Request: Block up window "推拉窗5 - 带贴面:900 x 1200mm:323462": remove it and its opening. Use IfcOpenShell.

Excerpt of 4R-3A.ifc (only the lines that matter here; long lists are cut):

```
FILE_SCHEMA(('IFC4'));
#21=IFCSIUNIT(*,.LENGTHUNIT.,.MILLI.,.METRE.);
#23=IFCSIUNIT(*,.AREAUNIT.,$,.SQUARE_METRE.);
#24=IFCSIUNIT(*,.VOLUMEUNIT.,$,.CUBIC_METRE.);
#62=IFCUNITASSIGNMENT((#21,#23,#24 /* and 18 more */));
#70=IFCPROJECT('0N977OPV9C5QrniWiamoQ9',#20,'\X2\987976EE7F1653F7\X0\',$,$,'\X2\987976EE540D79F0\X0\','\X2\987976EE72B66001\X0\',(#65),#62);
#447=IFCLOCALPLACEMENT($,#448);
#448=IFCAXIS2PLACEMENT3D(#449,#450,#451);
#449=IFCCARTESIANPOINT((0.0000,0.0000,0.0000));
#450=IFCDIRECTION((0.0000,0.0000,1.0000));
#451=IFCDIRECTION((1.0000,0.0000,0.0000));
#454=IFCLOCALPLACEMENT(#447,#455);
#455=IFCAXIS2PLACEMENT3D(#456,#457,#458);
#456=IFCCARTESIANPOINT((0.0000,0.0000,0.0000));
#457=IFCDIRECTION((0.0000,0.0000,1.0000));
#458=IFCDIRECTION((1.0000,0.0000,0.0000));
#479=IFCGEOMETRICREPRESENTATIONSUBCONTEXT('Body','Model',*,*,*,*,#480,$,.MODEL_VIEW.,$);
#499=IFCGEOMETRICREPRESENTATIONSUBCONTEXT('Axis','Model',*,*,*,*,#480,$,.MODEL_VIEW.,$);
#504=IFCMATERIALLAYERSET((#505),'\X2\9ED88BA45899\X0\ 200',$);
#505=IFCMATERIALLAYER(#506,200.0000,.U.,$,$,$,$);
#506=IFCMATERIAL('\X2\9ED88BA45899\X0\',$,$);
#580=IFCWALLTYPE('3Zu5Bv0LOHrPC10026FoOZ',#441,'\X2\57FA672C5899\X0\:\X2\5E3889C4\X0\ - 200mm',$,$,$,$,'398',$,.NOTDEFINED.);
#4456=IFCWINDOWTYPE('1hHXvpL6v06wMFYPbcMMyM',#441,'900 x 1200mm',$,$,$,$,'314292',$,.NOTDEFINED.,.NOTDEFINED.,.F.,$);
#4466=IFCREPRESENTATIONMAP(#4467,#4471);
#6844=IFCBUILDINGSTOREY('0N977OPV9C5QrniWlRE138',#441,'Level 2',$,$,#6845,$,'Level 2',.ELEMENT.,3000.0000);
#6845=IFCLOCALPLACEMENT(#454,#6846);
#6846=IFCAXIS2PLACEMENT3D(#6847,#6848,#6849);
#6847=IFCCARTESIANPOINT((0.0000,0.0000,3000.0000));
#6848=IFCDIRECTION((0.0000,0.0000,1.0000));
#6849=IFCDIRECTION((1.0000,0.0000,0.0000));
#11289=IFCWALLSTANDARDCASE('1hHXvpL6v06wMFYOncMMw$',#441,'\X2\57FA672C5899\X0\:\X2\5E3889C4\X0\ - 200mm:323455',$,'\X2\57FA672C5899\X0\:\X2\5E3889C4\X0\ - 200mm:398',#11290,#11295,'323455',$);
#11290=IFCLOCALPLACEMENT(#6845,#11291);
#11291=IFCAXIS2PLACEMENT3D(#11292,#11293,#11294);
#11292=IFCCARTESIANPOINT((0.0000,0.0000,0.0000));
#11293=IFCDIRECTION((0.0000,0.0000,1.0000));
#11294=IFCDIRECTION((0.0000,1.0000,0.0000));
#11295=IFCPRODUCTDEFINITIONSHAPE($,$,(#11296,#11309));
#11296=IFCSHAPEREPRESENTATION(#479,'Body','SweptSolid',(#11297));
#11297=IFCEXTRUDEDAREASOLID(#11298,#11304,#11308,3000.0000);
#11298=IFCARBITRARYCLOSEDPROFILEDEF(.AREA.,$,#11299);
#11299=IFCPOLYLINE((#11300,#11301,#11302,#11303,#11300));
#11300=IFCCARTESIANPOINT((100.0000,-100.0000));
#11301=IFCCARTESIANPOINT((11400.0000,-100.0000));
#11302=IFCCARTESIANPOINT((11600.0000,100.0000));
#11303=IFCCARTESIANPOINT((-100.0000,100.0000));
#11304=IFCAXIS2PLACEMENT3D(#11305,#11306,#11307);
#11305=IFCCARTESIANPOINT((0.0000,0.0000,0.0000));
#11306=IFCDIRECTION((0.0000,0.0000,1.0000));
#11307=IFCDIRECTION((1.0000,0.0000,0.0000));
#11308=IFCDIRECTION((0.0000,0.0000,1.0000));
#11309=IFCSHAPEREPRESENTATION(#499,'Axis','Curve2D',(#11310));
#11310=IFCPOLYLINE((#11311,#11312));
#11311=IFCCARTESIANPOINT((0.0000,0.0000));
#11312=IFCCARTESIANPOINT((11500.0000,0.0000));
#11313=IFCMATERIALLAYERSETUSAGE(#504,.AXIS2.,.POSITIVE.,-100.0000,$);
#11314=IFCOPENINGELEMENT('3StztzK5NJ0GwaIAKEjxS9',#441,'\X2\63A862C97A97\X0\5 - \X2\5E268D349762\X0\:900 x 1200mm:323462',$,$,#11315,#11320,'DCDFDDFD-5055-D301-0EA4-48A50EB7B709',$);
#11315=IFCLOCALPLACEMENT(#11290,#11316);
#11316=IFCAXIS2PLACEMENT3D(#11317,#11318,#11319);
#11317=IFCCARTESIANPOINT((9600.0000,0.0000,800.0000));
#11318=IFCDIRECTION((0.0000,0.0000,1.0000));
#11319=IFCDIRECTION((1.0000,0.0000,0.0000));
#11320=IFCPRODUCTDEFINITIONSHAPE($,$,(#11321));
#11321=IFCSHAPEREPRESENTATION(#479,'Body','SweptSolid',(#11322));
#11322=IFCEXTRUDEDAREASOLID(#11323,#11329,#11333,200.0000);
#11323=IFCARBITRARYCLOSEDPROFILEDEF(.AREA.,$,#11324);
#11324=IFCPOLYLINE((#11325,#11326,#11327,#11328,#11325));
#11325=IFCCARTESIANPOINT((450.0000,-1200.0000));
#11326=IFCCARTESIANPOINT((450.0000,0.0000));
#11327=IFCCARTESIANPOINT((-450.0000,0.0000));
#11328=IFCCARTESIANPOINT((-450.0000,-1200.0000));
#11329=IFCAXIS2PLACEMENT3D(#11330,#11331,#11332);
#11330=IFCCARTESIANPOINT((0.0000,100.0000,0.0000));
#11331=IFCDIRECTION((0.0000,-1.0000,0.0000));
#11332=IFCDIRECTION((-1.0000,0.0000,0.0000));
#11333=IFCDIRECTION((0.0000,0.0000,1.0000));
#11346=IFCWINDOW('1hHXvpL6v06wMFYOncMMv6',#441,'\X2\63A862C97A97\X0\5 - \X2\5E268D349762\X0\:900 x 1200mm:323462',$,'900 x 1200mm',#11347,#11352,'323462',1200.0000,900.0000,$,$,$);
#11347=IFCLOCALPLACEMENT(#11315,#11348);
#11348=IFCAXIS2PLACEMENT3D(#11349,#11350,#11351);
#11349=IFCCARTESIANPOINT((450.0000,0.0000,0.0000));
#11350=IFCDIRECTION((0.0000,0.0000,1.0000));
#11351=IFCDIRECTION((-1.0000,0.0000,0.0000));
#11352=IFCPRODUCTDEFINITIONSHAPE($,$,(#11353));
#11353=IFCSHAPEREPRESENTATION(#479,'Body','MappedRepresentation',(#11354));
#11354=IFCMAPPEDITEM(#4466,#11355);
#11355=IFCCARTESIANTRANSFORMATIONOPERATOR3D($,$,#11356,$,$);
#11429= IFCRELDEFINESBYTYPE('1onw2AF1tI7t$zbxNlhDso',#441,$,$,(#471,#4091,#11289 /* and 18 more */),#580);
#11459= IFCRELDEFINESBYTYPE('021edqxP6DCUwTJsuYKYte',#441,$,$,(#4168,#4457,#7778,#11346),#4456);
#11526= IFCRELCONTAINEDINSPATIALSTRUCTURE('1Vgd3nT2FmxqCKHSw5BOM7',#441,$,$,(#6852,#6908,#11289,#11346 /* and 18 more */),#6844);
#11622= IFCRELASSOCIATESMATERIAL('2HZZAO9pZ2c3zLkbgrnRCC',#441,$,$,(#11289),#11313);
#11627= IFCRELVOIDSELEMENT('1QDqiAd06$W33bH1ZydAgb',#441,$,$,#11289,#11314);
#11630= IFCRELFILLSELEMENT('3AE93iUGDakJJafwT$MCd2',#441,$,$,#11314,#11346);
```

```python
import ifcopenshell
import ifcopenshell.api.feature
import ifcopenshell.api.root
import ifcopenshell.geom
import ifcopenshell.util.shape

model = ifcopenshell.open("4R-3A.ifc")
settings = ifcopenshell.geom.settings()


def volume(element):
    """Net volume in cubic metres, openings subtracted."""
    shape = ifcopenshell.geom.create_shape(settings, element)
    return ifcopenshell.util.shape.get_volume(shape.geometry)


window = model.by_guid("1hHXvpL6v06wMFYOncMMv6")
opening = window.FillsVoids[0].RelatingOpeningElement
wall = opening.VoidsElements[0].RelatingBuildingElement
before = volume(wall)

ifcopenshell.api.root.remove_product(model, product=window)
ifcopenshell.api.feature.remove_feature(model, feature=opening)

after = volume(wall)

print(f"wall volume {before:.3f} -> {after:.3f} m3")

model.write("4R-3A-out.ifc")
```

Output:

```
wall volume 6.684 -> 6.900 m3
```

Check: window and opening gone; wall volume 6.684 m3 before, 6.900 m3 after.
